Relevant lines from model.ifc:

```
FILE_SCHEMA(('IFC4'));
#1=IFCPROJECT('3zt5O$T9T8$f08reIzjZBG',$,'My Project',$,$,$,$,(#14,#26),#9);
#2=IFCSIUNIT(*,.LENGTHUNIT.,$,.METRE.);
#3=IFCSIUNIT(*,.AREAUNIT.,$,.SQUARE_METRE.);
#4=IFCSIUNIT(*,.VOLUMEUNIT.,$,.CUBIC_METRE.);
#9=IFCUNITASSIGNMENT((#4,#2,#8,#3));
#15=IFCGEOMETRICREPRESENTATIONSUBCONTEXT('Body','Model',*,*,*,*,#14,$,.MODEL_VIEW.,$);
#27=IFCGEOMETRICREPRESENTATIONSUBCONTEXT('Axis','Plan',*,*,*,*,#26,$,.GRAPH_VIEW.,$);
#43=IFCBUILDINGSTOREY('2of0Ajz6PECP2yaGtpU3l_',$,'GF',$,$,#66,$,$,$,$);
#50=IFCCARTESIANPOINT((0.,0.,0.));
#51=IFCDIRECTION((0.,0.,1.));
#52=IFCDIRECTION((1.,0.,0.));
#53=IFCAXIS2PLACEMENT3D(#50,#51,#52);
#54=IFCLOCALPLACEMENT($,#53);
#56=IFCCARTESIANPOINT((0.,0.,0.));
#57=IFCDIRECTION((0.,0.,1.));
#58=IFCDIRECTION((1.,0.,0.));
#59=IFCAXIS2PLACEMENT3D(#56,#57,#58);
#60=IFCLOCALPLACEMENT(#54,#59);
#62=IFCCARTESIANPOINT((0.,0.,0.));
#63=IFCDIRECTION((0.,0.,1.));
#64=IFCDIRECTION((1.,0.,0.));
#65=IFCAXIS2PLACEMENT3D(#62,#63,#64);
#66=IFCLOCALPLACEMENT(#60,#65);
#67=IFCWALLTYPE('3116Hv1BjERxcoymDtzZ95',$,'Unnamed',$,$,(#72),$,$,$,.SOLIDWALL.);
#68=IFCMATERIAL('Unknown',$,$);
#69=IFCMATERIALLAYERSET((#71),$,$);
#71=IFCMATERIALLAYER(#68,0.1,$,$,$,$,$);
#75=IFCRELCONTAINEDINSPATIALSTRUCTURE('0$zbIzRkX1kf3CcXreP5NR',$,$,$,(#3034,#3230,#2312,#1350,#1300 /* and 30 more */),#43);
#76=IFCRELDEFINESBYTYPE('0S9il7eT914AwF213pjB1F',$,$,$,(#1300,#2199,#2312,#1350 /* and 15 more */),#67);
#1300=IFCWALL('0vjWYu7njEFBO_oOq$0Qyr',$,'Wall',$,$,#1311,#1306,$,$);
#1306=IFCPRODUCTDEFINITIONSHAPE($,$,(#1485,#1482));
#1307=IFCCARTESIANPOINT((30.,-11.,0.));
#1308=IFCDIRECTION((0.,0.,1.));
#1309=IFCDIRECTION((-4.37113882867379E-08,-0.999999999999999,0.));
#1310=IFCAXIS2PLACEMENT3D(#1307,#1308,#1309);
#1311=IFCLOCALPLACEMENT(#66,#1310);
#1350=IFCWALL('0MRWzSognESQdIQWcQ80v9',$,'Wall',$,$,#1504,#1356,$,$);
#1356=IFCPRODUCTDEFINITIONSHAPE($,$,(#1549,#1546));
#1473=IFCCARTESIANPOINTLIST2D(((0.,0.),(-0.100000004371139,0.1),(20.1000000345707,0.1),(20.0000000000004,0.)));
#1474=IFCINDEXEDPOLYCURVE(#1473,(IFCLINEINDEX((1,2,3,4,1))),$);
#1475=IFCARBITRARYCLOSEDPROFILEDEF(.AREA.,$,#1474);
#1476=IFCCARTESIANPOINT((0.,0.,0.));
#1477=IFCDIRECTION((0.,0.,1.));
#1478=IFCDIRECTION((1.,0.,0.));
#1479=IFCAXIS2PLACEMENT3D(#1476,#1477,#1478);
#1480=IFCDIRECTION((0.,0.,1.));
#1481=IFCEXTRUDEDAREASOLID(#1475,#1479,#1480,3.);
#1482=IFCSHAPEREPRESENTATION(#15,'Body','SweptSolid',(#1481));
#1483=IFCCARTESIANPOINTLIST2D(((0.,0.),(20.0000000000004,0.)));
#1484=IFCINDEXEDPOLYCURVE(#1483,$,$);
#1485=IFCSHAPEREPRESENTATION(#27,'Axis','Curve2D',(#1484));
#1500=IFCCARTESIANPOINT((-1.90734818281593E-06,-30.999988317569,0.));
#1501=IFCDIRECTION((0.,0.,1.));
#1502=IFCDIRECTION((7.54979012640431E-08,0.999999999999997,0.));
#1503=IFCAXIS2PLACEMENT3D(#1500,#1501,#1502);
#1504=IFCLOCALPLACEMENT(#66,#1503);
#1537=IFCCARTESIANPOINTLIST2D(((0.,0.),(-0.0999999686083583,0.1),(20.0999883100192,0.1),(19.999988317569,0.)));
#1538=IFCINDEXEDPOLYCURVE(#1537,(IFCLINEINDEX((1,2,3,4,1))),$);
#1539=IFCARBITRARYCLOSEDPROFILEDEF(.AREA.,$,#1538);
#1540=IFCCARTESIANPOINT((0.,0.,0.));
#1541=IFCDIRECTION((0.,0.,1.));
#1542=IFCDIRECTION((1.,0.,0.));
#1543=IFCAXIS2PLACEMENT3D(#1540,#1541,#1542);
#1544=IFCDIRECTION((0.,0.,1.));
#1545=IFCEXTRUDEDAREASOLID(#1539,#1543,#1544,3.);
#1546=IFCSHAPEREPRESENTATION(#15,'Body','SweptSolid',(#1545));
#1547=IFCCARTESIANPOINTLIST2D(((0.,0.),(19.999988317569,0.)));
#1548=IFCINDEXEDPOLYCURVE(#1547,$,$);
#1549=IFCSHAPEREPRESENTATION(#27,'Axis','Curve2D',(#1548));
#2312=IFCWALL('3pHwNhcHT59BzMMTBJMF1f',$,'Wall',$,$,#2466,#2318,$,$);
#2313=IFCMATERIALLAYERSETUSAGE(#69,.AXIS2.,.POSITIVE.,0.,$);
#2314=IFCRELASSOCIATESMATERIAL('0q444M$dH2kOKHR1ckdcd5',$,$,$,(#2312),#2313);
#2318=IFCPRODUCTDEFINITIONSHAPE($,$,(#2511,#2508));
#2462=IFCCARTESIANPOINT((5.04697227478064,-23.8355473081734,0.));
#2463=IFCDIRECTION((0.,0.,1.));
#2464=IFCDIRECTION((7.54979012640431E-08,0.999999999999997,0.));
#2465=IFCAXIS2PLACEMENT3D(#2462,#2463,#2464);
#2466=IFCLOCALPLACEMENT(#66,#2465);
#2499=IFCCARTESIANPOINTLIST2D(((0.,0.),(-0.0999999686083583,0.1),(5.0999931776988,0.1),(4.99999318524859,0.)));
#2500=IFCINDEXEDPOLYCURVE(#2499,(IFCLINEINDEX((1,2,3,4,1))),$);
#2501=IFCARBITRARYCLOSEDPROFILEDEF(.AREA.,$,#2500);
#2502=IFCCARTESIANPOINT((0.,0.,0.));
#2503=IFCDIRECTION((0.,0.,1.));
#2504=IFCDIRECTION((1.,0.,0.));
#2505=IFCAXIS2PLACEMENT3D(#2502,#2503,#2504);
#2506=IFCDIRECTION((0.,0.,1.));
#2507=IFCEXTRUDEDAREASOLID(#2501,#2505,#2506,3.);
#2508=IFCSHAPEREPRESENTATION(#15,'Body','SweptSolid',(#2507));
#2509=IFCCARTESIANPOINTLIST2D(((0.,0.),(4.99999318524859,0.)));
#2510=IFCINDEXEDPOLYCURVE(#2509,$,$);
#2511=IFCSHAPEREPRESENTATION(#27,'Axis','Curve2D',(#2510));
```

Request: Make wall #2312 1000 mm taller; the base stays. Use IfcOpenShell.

```python
import ifcopenshell
import ifcopenshell.geom
import ifcopenshell.util.representation
import ifcopenshell.util.shape

model = ifcopenshell.open("model.ifc")
settings = ifcopenshell.geom.settings()


def volume(element):
    """Net volume in cubic metres, openings subtracted."""
    shape = ifcopenshell.geom.create_shape(settings, element)
    return ifcopenshell.util.shape.get_volume(shape.geometry)


wall = model.by_guid("3pHwNhcHT59BzMMTBJMF1f")
before = volume(wall)

body = ifcopenshell.util.representation.get_representation(wall, "Model", "Body")
solid = body.Items[0]
old_height = solid.Depth
solid.Depth += 1.0
after = volume(wall)

print(f"height {old_height:g} -> {solid.Depth:g}, volume {before:.3f} -> {after:.3f} m3")

model.write("model_rev.ifc")
```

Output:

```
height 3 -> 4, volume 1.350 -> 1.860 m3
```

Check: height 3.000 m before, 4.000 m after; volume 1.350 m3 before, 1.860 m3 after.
